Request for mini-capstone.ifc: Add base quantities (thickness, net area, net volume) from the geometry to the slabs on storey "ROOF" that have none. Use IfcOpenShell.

First a look at what the model holds.

```python
import ifcopenshell
import ifcopenshell.util.element
import ifcopenshell.util.unit

model = ifcopenshell.open("mini-capstone.ifc")
print(model.schema)
for unit_type in ("LENGTHUNIT", "AREAUNIT", "VOLUMEUNIT"):
    print(unit_type, ifcopenshell.util.unit.calculate_unit_scale(model, unit_type))
storey = next(s for s in model.by_type("IfcBuildingStorey") if s.Name == "ROOF")
slabs = [e for e in ifcopenshell.util.element.get_decomposition(storey) if e.is_a("IfcSlab")]
for e in sorted(slabs, key=lambda e: e.id()):
    print(e.id(), e.is_a(), e.Name, list(ifcopenshell.util.element.get_psets(e, qtos_only=True)), sep=" | ")
```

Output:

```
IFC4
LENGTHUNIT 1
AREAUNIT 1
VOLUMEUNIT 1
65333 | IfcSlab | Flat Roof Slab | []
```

```python
import ifcopenshell
import ifcopenshell.api.pset
import ifcopenshell.geom
import ifcopenshell.util.element
import ifcopenshell.util.shape
import ifcopenshell.util.unit

model = ifcopenshell.open("mini-capstone.ifc")
unit_scale = ifcopenshell.util.unit.calculate_unit_scale(model)
area_scale = ifcopenshell.util.unit.calculate_unit_scale(model, "AREAUNIT")
volume_scale = ifcopenshell.util.unit.calculate_unit_scale(model, "VOLUMEUNIT")
settings = ifcopenshell.geom.settings()

storey = next(s for s in model.by_type("IfcBuildingStorey") if s.Name == "ROOF")
slabs = [e for e in ifcopenshell.util.element.get_decomposition(storey) if e.is_a("IfcSlab")]

for e in sorted(slabs, key=lambda e: e.id()):
    if ifcopenshell.util.element.get_psets(e, qtos_only=True, should_inherit=False):
        continue
    # Geometry comes back in metres, in the element's own axes.
    shape = ifcopenshell.geom.create_shape(settings, e)
    values = {
        "Width": ifcopenshell.util.shape.get_z(shape.geometry) / unit_scale,
        "NetArea": ifcopenshell.util.shape.get_footprint_area(shape.geometry) / area_scale,
        "NetVolume": ifcopenshell.util.shape.get_volume(shape.geometry) / volume_scale,
    }
    qto = ifcopenshell.api.pset.add_qto(model, product=e, name="Qto_SlabBaseQuantities")
    ifcopenshell.api.pset.edit_qto(model, qto=qto, properties=values)
    print(e.id(), {k: round(v, 3) for k, v in values.items()})

model.write("mini-capstone-out.ifc")
```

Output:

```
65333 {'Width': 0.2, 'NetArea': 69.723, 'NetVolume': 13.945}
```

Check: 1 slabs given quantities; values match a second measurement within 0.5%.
